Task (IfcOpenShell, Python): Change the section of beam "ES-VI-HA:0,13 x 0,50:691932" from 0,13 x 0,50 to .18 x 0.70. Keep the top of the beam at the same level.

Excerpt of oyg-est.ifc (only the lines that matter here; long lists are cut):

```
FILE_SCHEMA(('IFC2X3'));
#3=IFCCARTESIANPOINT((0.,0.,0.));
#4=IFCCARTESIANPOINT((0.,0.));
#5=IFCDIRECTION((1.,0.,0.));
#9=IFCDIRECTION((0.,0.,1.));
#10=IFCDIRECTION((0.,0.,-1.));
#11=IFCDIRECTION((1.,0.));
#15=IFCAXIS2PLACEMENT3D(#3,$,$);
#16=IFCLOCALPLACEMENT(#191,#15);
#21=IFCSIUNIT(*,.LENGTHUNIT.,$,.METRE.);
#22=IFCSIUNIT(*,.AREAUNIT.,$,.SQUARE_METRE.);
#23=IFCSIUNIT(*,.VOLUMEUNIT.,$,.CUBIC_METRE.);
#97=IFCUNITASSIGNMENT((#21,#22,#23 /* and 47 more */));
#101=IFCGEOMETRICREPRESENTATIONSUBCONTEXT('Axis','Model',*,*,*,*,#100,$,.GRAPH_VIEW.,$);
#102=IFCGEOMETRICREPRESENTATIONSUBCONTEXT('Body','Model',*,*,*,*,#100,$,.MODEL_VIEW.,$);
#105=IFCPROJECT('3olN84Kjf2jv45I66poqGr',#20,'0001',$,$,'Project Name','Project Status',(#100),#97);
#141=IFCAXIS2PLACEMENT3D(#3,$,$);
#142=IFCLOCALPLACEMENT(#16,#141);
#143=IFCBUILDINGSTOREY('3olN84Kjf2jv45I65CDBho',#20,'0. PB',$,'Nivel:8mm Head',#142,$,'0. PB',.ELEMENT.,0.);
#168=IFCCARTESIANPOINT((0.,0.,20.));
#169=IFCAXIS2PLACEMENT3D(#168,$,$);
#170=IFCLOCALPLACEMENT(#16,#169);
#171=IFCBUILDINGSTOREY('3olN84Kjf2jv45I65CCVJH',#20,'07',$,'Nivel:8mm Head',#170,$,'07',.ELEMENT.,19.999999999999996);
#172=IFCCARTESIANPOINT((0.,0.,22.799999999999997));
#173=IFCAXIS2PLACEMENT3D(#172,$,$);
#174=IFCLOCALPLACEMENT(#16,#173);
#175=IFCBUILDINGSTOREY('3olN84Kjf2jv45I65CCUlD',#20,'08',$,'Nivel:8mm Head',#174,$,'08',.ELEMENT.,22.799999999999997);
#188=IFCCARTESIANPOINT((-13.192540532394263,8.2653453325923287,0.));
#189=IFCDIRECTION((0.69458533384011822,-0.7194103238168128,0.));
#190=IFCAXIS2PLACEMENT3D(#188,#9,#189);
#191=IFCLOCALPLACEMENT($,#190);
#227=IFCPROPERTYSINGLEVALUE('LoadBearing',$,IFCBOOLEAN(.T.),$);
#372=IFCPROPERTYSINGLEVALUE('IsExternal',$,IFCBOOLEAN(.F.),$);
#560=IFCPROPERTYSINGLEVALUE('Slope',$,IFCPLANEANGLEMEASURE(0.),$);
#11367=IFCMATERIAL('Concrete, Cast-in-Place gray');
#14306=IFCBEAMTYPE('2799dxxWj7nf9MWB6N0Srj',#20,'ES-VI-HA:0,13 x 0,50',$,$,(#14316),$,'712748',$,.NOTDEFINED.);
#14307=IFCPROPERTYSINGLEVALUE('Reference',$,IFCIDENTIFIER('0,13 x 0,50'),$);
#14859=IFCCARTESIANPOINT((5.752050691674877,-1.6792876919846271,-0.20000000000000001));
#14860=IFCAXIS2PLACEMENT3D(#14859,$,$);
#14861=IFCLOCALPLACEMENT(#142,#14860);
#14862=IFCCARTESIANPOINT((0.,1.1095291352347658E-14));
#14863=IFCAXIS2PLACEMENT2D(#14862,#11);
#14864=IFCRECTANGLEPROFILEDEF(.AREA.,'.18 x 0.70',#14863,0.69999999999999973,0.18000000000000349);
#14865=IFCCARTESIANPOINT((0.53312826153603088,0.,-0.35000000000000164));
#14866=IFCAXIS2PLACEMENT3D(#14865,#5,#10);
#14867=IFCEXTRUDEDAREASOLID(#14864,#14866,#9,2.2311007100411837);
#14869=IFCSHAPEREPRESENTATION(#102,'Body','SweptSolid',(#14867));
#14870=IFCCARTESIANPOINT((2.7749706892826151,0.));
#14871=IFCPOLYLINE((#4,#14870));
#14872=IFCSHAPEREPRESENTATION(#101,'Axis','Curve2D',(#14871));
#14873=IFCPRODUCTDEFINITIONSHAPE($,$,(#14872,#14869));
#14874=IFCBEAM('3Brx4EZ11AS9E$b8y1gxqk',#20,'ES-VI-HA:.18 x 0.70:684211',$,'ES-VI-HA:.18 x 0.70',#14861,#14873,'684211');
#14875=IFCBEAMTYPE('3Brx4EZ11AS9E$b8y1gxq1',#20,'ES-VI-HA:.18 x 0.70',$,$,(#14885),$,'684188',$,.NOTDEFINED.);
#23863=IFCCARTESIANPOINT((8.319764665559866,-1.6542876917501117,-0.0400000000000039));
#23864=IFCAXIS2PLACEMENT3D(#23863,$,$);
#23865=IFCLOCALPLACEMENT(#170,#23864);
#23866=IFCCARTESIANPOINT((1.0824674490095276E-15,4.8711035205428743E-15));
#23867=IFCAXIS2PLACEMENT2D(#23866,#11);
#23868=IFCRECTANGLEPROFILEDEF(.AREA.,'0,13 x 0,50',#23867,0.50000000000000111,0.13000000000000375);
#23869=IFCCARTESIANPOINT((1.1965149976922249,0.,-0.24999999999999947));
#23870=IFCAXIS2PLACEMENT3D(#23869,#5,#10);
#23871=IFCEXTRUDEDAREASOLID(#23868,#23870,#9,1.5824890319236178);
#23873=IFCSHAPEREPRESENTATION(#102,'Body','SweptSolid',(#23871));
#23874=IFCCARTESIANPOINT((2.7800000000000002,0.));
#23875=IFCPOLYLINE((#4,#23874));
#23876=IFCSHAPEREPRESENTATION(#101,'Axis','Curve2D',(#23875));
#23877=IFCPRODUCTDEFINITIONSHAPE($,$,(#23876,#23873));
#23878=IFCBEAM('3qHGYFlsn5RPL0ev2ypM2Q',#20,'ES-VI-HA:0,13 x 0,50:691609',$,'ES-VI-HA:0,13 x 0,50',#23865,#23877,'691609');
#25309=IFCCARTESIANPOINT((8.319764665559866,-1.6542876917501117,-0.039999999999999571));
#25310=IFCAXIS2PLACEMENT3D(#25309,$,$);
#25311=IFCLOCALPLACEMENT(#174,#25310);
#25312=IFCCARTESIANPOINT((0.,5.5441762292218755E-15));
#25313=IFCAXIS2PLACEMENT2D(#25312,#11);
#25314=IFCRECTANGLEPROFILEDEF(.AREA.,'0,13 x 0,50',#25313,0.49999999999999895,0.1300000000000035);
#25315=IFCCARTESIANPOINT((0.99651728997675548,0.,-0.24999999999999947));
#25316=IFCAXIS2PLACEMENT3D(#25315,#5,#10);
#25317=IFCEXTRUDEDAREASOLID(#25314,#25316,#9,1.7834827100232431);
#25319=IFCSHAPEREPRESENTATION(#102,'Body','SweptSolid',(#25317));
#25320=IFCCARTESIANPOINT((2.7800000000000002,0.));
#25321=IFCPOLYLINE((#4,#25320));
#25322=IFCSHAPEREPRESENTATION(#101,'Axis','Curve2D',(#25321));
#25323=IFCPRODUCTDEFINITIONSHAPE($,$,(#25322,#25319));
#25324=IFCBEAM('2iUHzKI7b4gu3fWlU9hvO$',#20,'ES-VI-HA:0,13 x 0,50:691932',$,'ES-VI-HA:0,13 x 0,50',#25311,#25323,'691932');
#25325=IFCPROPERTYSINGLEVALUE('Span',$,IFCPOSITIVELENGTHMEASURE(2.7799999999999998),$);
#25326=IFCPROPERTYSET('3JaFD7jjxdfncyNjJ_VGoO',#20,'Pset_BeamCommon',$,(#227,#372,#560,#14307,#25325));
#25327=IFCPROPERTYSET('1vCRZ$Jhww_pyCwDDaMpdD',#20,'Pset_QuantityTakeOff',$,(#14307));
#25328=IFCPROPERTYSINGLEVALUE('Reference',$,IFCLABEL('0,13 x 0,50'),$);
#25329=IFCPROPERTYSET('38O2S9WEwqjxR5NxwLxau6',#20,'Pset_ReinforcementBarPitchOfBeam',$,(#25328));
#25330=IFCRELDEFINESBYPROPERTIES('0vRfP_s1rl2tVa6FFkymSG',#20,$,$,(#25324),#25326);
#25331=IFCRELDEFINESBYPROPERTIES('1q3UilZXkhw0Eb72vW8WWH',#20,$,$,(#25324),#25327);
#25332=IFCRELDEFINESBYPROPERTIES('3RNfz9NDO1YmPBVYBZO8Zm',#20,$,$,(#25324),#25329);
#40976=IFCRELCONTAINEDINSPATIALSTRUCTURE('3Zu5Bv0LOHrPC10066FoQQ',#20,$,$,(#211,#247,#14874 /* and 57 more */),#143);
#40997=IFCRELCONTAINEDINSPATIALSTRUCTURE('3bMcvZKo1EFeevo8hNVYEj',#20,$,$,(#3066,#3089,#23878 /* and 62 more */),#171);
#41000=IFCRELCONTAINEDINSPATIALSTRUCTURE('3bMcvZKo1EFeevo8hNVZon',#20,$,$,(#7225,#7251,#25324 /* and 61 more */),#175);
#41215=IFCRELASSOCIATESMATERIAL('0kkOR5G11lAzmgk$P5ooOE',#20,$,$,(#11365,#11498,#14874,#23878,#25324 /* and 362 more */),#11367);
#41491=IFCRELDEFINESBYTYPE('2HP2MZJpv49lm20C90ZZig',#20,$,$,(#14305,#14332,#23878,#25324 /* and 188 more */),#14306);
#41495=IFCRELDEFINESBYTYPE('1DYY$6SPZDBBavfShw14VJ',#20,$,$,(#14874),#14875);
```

```python
import ifcopenshell
import ifcopenshell.api.pset
import ifcopenshell.api.type
import ifcopenshell.util.element
import ifcopenshell.util.representation

model = ifcopenshell.open("oyg-est.ifc")

member = model.by_guid("2iUHzKI7b4gu3fWlU9hvO$")
source = next(p for p in model.by_type("IfcRectangleProfileDef") if p.ProfileName == ".18 x 0.70")

body = ifcopenshell.util.representation.get_representation(member, "Model", "Body")
solid = body.Items[0]
old_profile = solid.SweptArea

# Copy the section's sizes but keep this member's own profile position.
profile = ifcopenshell.util.element.copy(model, source)
# Profiles are centred, so shift by half the change in depth to hold the top.
shift = (old_profile.XDim - profile.XDim) / 2
x, y = old_profile.Position.Location.Coordinates
up = (-1.0, 0.0)  # upwards, in the solid's own plane
location = model.createIfcCartesianPoint((x + up[0] * shift, y + up[1] * shift))
profile.Position = model.createIfcAxis2Placement2D(location, old_profile.Position.RefDirection)
solid.SweptArea = profile
if not model.get_total_inverses(old_profile):
    ifcopenshell.util.element.remove_deep2(model, old_profile)

new_type = model.by_guid("3Brx4EZ11AS9E$b8y1gxq1")
ifcopenshell.api.type.assign_type(
    model, related_objects=[member], relating_type=new_type, should_map_representations=False
)
member.Name = member.Name.replace("0,13 x 0,50", ".18 x 0.70")
member.ObjectType = "ES-VI-HA:.18 x 0.70"
pset = model.by_id(ifcopenshell.util.element.get_pset(member, "Pset_BeamCommon", should_inherit=False)["id"])
ifcopenshell.api.pset.edit_pset(model, pset=pset, properties={"Reference": ".18 x 0.70"})
pset = model.by_id(ifcopenshell.util.element.get_pset(member, "Pset_QuantityTakeOff", should_inherit=False)["id"])
ifcopenshell.api.pset.edit_pset(model, pset=pset, properties={"Reference": ".18 x 0.70"})
pset = model.by_id(ifcopenshell.util.element.get_pset(member, "Pset_ReinforcementBarPitchOfBeam", should_inherit=False)["id"])
ifcopenshell.api.pset.edit_pset(model, pset=pset, properties={"Reference": ".18 x 0.70"})

print(solid.SweptArea)

model.write("oyg-est_v2.ifc")
```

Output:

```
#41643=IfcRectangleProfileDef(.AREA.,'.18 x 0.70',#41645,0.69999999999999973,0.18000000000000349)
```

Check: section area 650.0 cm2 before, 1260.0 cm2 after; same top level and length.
